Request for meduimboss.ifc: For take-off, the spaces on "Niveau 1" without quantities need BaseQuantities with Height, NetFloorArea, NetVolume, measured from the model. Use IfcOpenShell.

First a look at what the model holds.

```python
import ifcopenshell
import ifcopenshell.util.element
import ifcopenshell.util.unit

model = ifcopenshell.open("meduimboss.ifc")
print(model.schema)
for unit_type in ("LENGTHUNIT", "AREAUNIT", "VOLUMEUNIT"):
    print(unit_type, ifcopenshell.util.unit.calculate_unit_scale(model, unit_type))
storey = next(s for s in model.by_type("IfcBuildingStorey") if s.Name == "Niveau 1")
spaces = [e for e in ifcopenshell.util.element.get_decomposition(storey) if e.is_a("IfcSpace")]
for e in sorted(spaces, key=lambda e: e.id()):
    print(e.id(), e.is_a(), e.Name, list(ifcopenshell.util.element.get_psets(e, qtos_only=True)), sep=" | ")
```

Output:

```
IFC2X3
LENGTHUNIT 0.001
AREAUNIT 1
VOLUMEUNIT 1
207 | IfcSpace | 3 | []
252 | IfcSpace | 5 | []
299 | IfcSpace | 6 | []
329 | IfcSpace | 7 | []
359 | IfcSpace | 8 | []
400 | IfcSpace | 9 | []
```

```python
import ifcopenshell
import ifcopenshell.api.pset
import ifcopenshell.geom
import ifcopenshell.util.element
import ifcopenshell.util.shape
import ifcopenshell.util.unit

model = ifcopenshell.open("meduimboss.ifc")
unit_scale = ifcopenshell.util.unit.calculate_unit_scale(model)
area_scale = ifcopenshell.util.unit.calculate_unit_scale(model, "AREAUNIT")
volume_scale = ifcopenshell.util.unit.calculate_unit_scale(model, "VOLUMEUNIT")
settings = ifcopenshell.geom.settings()

storey = next(s for s in model.by_type("IfcBuildingStorey") if s.Name == "Niveau 1")
spaces = [e for e in ifcopenshell.util.element.get_decomposition(storey) if e.is_a("IfcSpace")]

for e in sorted(spaces, key=lambda e: e.id()):
    if ifcopenshell.util.element.get_psets(e, qtos_only=True, should_inherit=False):
        continue
    # Geometry comes back in metres, in the element's own axes.
    shape = ifcopenshell.geom.create_shape(settings, e)
    values = {
        "Height": ifcopenshell.util.shape.get_z(shape.geometry) / unit_scale,
        "NetFloorArea": ifcopenshell.util.shape.get_footprint_area(shape.geometry) / area_scale,
        "NetVolume": ifcopenshell.util.shape.get_volume(shape.geometry) / volume_scale,
    }
    qto = ifcopenshell.api.pset.add_qto(model, product=e, name="BaseQuantities")
    ifcopenshell.api.pset.edit_qto(model, qto=qto, properties=values)
    print(e.id(), {k: round(v, 3) for k, v in values.items()})

model.write("meduimboss_edited.ifc")
```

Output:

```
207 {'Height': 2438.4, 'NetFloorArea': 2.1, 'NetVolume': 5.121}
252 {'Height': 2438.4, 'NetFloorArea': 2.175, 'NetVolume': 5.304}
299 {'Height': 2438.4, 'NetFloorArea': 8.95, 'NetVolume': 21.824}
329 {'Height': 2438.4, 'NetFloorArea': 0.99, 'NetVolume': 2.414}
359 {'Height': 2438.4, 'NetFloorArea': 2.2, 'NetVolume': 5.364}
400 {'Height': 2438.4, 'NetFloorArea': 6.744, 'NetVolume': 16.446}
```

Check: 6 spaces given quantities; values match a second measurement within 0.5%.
